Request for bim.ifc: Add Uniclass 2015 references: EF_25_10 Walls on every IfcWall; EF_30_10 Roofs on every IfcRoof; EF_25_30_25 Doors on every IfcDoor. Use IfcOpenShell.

First a look at what the model holds.

```python
import ifcopenshell

model = ifcopenshell.open("bim.ifc")
print(model.schema)
print("classifications:", [c.Name for c in model.by_type("IfcClassification")])
for ifc_class in ("IfcDoor", "IfcRoof", "IfcStair", "IfcWall", "IfcWindow"):
    print(ifc_class, len(model.by_type(ifc_class)))
```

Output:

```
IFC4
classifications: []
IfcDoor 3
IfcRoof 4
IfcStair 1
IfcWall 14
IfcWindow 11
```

```python
import ifcopenshell
import ifcopenshell.api.classification

model = ifcopenshell.open("bim.ifc")

system = ifcopenshell.api.classification.add_classification(model, classification="Uniclass 2015")

codes = {
    "IfcWall": ("EF_25_10", "Walls"),
    "IfcRoof": ("EF_30_10", "Roofs"),
    "IfcDoor": ("EF_25_30_25", "Doors"),
}
for ifc_class, (code, name) in codes.items():
    products = model.by_type(ifc_class)
    ifcopenshell.api.classification.add_reference(
        model, products=products, classification=system, identification=code, name=name
    )
    print(code, len(products))

model.write("bim_updated.ifc")
```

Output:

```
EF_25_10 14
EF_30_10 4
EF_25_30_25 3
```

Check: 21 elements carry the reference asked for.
